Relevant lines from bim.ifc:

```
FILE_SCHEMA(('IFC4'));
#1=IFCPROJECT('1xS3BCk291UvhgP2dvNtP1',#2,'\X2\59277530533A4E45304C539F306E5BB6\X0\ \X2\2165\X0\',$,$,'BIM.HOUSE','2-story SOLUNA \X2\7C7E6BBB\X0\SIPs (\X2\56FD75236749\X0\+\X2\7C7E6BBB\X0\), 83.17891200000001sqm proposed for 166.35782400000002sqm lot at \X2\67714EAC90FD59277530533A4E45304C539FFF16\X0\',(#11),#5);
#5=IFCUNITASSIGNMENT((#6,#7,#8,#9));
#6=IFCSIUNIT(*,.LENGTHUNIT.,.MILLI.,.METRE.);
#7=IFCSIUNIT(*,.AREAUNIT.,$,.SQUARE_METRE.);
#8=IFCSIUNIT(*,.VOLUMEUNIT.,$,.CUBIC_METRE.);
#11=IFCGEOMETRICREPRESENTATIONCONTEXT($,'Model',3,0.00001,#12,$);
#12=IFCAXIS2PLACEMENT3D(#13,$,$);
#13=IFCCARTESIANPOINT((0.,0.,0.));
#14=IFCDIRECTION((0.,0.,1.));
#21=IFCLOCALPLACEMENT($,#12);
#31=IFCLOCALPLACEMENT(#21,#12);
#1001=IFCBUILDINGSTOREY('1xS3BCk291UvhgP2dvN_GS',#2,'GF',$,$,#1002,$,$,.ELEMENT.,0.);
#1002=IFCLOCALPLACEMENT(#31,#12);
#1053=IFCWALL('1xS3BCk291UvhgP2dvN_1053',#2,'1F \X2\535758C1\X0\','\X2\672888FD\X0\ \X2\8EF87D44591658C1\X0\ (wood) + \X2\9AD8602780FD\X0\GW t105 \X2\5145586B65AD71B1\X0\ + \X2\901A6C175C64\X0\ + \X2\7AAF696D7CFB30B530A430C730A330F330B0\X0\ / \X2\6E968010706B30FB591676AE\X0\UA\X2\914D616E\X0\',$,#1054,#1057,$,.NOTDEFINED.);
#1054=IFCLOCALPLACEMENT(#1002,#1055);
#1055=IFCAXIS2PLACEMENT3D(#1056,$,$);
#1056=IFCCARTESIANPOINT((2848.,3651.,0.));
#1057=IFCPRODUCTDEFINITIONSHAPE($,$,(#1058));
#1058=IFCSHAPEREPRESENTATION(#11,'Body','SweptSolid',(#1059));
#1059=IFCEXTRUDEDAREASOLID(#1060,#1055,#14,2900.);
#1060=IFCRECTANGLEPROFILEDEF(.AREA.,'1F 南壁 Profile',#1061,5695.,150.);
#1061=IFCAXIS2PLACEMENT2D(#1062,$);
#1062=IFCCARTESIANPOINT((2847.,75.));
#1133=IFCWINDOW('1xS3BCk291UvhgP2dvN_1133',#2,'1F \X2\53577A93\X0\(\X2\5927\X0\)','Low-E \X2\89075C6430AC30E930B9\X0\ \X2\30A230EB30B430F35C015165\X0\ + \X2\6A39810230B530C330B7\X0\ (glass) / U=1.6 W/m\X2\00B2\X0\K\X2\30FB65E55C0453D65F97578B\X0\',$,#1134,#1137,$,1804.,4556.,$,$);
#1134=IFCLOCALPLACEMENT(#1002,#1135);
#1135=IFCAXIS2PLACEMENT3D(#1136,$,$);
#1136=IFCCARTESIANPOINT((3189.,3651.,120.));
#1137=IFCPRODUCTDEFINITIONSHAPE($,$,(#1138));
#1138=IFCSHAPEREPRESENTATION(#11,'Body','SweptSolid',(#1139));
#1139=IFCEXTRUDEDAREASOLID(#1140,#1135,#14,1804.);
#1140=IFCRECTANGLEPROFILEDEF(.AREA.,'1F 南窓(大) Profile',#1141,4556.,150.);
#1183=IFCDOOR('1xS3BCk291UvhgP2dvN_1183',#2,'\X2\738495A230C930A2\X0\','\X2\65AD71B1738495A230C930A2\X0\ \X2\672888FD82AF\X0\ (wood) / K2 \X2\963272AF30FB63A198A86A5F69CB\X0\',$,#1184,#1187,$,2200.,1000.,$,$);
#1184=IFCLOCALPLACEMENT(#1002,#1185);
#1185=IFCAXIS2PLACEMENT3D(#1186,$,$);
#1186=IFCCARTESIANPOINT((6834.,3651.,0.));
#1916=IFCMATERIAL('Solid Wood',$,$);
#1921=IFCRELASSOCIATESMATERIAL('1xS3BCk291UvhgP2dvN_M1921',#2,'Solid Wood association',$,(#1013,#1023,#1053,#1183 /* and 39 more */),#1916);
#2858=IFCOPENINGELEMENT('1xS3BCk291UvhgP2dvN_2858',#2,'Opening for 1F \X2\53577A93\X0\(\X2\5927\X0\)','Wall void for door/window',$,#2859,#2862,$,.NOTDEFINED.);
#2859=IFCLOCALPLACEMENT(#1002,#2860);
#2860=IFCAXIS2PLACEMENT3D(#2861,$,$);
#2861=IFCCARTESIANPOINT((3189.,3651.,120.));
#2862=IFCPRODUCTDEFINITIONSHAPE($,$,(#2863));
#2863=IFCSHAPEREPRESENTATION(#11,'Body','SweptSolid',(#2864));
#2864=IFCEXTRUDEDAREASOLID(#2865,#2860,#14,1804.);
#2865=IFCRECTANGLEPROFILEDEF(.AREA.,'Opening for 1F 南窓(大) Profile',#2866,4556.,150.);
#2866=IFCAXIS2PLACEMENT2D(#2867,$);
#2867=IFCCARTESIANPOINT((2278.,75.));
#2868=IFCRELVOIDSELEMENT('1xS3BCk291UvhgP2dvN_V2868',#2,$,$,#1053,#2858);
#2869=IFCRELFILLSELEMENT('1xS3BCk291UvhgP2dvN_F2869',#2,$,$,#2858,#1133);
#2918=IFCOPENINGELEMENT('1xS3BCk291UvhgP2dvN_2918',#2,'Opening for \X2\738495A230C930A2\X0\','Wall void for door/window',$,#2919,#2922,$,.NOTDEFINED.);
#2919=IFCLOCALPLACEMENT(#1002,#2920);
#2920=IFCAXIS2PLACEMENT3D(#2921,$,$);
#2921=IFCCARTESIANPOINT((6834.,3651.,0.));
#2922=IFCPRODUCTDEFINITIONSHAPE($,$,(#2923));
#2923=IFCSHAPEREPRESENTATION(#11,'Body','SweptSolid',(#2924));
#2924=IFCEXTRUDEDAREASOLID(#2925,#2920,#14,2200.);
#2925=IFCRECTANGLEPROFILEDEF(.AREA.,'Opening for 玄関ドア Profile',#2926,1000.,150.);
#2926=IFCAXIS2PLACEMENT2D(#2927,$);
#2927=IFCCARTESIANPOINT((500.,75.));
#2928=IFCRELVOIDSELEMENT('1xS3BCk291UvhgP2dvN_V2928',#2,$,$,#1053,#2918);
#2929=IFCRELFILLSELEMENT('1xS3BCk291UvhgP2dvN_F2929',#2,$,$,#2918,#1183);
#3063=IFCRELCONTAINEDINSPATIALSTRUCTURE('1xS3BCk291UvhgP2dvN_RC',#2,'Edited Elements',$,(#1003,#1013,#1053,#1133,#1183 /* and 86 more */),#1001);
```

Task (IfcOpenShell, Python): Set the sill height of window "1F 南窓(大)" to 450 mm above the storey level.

```python
import numpy as np
import ifcopenshell
import ifcopenshell.api.geometry
import ifcopenshell.geom
import ifcopenshell.util.element
import ifcopenshell.util.placement
import ifcopenshell.util.shape
import ifcopenshell.util.unit

model = ifcopenshell.open("bim.ifc")
unit_scale = ifcopenshell.util.unit.calculate_unit_scale(model)

window = model.by_id(1133)
opening = window.FillsVoids[0].RelatingOpeningElement
storey = ifcopenshell.util.element.get_container(window, ifc_class="IfcBuildingStorey")
level = ifcopenshell.util.placement.get_local_placement(storey.ObjectPlacement)[2, 3]

# The opening's origin need not be at the sill, so measure its lowest point.
shape = ifcopenshell.geom.create_shape(ifcopenshell.geom.settings(), opening)
bottom = ifcopenshell.util.shape.get_shape_bottom_elevation(shape, shape.geometry) / unit_scale
dz = level + 0.45 / unit_scale - bottom

shift = np.array([0.0, 0.0, dz])
# The window is not placed relative to its opening, so move both.
for product in (opening, window):
    matrix = ifcopenshell.util.placement.get_local_placement(product.ObjectPlacement)
    matrix[:3, 3] += shift
    ifcopenshell.api.geometry.edit_object_placement(model, product=product, matrix=matrix, is_si=False)

print(f"moved by {dz * unit_scale:+.3f} m")

model.write("bim_updated.ifc")
```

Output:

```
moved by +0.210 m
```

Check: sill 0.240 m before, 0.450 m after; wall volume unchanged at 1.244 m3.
